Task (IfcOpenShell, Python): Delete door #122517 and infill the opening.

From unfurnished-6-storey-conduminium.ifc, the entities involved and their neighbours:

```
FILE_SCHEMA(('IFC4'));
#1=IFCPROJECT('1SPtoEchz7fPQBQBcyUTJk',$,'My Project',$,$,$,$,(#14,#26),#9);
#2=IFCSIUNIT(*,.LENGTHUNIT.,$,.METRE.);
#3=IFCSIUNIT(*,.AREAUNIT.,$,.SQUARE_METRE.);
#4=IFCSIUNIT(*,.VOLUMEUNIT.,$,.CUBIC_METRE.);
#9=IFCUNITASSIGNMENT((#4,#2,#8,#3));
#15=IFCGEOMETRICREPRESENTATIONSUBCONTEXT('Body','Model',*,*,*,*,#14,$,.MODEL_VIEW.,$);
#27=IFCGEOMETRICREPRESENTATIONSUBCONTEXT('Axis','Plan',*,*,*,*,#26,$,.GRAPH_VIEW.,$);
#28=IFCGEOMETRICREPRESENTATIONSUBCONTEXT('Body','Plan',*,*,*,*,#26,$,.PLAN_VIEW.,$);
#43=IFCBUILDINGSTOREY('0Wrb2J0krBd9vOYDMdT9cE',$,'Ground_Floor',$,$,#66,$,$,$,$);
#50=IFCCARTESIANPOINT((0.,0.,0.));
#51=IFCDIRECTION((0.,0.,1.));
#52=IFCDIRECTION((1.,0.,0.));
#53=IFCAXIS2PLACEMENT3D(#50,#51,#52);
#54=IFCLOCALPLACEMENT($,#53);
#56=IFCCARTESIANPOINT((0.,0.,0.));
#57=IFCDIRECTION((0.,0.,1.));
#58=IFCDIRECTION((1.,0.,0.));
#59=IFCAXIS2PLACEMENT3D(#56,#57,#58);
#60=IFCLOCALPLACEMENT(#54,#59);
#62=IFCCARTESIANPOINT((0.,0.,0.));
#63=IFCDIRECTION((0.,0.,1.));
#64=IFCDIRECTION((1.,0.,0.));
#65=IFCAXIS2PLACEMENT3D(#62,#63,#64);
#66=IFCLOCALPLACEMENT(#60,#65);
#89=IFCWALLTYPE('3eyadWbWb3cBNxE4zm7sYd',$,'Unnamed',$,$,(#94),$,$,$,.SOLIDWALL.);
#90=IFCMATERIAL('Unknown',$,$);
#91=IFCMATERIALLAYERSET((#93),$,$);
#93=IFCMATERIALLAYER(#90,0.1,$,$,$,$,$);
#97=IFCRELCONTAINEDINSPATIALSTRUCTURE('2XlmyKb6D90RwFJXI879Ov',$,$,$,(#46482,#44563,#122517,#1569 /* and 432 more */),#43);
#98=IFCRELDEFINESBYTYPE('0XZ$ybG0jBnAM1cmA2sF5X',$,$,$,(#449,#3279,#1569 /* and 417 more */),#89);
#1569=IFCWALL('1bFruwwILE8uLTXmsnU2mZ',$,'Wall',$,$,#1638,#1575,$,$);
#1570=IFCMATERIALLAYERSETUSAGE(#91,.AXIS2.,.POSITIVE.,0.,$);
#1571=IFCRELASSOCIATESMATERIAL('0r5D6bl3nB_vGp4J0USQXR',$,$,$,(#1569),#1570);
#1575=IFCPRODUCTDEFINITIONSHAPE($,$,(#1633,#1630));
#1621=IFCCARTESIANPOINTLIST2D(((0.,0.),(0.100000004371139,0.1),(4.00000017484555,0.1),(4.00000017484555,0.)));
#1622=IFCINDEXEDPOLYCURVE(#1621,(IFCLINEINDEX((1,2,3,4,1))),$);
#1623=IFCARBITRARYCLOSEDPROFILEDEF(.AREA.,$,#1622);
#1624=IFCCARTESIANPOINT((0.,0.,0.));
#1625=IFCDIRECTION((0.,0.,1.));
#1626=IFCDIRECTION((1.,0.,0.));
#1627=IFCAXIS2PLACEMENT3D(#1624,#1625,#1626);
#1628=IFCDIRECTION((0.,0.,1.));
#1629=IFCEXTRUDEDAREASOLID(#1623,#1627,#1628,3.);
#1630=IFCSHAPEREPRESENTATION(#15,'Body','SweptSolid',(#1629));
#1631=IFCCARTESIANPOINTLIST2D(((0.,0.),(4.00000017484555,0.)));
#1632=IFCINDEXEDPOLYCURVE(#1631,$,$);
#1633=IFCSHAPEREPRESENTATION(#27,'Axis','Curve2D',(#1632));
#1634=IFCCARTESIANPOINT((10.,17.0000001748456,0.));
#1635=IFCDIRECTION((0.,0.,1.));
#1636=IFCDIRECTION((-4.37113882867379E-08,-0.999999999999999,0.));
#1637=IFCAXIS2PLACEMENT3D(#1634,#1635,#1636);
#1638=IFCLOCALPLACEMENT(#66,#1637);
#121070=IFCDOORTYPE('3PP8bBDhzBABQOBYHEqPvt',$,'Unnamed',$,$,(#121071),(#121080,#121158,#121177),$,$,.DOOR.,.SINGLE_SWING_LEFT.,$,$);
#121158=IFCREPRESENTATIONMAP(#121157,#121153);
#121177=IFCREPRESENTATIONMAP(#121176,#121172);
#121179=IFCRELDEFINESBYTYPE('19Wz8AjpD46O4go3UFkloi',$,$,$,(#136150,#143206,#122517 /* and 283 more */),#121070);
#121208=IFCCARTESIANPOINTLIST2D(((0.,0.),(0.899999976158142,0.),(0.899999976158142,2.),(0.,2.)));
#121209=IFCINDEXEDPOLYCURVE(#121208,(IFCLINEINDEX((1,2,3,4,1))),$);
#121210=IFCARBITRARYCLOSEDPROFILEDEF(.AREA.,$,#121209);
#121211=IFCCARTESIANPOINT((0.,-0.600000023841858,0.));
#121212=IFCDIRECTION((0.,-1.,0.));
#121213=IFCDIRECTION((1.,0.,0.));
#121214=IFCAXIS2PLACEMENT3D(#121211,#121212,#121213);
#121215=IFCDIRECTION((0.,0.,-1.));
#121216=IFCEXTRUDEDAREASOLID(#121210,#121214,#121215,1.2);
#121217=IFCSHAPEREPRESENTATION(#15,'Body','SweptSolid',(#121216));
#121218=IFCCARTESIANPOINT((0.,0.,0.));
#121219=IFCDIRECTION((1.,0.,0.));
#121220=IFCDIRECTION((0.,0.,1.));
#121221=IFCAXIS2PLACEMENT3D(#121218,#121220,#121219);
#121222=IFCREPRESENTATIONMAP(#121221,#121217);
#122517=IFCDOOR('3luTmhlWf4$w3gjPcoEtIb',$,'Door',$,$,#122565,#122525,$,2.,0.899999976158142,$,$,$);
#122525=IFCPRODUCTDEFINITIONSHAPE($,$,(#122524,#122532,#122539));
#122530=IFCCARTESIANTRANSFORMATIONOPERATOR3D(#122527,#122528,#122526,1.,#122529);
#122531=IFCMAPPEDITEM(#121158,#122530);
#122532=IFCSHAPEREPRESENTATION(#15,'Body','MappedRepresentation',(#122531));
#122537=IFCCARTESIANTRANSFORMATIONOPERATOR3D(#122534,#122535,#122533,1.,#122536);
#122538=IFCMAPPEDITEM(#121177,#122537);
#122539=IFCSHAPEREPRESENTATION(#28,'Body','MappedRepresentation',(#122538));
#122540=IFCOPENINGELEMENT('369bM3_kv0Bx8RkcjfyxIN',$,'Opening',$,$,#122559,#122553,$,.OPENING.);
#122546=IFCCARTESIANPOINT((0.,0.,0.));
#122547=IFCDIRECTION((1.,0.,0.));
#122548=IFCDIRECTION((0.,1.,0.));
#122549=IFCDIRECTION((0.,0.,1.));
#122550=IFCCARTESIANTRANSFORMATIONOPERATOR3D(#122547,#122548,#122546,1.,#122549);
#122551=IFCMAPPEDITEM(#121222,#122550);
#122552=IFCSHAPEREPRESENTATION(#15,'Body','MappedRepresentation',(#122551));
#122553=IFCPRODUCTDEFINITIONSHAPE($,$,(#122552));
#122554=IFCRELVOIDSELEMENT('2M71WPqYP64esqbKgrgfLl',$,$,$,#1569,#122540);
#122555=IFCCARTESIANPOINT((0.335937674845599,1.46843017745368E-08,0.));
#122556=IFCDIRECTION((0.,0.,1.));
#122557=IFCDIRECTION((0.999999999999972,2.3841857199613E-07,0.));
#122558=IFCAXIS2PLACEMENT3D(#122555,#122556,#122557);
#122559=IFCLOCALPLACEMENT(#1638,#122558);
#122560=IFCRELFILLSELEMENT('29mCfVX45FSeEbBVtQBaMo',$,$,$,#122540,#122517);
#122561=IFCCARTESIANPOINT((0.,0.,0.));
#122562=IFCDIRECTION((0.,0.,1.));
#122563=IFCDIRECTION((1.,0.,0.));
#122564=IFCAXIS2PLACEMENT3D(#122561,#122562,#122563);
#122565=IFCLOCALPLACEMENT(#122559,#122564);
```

```python
import ifcopenshell
import ifcopenshell.api.feature
import ifcopenshell.api.root
import ifcopenshell.geom
import ifcopenshell.util.shape

model = ifcopenshell.open("unfurnished-6-storey-conduminium.ifc")
settings = ifcopenshell.geom.settings()


def volume(element):
    """Net volume in cubic metres, openings subtracted."""
    shape = ifcopenshell.geom.create_shape(settings, element)
    return ifcopenshell.util.shape.get_volume(shape.geometry)


door = model.by_guid("3luTmhlWf4$w3gjPcoEtIb")
opening = door.FillsVoids[0].RelatingOpeningElement
wall = opening.VoidsElements[0].RelatingBuildingElement
before = volume(wall)

ifcopenshell.api.root.remove_product(model, product=door)
ifcopenshell.api.feature.remove_feature(model, feature=opening)

after = volume(wall)

print(f"wall volume {before:.3f} -> {after:.3f} m3")

model.write("unfurnished-6-storey-conduminium_edited.ifc")
```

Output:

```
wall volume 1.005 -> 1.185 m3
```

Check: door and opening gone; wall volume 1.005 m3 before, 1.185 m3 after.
